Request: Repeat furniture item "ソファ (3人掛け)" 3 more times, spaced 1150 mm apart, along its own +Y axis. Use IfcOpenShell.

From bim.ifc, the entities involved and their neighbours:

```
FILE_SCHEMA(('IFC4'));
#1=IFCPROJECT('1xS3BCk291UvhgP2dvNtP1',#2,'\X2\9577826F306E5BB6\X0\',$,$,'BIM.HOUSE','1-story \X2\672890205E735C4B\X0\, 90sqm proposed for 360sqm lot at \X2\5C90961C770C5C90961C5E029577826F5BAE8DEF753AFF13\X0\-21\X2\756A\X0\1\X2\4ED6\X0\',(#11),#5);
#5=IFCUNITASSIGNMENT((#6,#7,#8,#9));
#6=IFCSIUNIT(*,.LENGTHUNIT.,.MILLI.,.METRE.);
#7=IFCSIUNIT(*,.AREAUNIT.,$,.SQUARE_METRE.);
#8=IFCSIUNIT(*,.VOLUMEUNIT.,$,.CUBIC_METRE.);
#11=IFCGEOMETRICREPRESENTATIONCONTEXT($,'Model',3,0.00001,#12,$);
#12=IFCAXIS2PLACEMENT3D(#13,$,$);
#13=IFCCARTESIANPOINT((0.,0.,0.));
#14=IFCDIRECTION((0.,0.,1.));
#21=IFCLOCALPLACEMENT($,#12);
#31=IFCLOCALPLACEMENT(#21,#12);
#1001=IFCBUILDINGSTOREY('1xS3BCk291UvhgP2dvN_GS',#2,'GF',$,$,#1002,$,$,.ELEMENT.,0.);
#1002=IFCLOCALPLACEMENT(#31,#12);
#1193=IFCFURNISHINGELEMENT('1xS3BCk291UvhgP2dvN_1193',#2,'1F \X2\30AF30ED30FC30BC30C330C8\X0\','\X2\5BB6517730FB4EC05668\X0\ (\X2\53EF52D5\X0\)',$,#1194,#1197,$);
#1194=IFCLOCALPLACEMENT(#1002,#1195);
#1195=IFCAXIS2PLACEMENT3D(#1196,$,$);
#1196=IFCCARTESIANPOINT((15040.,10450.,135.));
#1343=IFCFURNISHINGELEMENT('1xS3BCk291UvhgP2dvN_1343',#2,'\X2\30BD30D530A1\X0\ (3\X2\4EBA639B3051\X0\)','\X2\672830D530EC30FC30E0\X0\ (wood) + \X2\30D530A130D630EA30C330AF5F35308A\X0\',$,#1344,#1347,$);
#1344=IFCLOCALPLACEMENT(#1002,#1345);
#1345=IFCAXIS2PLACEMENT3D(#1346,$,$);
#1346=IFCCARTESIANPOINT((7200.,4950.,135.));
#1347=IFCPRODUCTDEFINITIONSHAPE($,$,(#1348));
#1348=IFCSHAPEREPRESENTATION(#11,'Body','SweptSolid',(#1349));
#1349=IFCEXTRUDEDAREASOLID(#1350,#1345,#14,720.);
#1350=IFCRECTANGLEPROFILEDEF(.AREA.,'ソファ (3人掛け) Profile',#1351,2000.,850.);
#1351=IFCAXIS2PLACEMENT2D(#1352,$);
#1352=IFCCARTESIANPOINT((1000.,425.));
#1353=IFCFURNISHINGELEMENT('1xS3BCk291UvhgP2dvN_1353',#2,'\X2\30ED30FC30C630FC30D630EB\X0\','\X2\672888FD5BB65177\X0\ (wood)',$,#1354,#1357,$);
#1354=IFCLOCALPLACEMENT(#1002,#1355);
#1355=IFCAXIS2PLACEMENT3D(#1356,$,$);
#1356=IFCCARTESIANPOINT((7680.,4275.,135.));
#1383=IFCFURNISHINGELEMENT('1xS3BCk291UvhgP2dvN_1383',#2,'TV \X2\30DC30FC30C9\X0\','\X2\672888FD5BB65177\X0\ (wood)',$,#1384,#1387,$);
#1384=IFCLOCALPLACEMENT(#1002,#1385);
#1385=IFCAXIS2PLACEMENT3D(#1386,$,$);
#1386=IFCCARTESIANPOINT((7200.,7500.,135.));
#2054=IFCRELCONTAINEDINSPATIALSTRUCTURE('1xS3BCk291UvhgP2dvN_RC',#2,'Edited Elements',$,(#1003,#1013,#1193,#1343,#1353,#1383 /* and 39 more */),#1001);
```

```python
import ifcopenshell
import ifcopenshell.api.geometry
import ifcopenshell.api.root
import ifcopenshell.util.element
import ifcopenshell.util.placement
import ifcopenshell.util.unit

model = ifcopenshell.open("bim.ifc")
unit_scale = ifcopenshell.util.unit.calculate_unit_scale(model)


def reuse_history(source, copy):
    """copy_class also copies each property set's owner history, people and application; keep the originals."""
    for rel in copy.IsDefinedBy:
        if rel.is_a("IfcRelDefinesByProperties") and (history := rel.RelatingPropertyDefinition.OwnerHistory):
            rel.RelatingPropertyDefinition.OwnerHistory = source.OwnerHistory
            ifcopenshell.util.element.remove_deep2(model, history)


source = model.by_guid("1xS3BCk291UvhgP2dvN_1343")
base = ifcopenshell.util.placement.get_local_placement(source.ObjectPlacement)
step = base[:3, 1] * 1.15 / unit_scale

for i in range(1, 4):
    copy = ifcopenshell.api.root.copy_class(model, product=source)
    copy.Representation = ifcopenshell.util.element.copy_deep(
        model, source.Representation, exclude=["IfcGeometricRepresentationContext", "IfcRepresentationMap"]
    )
    reuse_history(source, copy)
    matrix = base.copy()
    matrix[:3, 3] += i * step
    print("added at", matrix[:3, 3].round(3) + 0.0)
    ifcopenshell.api.geometry.edit_object_placement(model, product=copy, matrix=matrix, is_si=False)

model.write("bim_edited.ifc")
```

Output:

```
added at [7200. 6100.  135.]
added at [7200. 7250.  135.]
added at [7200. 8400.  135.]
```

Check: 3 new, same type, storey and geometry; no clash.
